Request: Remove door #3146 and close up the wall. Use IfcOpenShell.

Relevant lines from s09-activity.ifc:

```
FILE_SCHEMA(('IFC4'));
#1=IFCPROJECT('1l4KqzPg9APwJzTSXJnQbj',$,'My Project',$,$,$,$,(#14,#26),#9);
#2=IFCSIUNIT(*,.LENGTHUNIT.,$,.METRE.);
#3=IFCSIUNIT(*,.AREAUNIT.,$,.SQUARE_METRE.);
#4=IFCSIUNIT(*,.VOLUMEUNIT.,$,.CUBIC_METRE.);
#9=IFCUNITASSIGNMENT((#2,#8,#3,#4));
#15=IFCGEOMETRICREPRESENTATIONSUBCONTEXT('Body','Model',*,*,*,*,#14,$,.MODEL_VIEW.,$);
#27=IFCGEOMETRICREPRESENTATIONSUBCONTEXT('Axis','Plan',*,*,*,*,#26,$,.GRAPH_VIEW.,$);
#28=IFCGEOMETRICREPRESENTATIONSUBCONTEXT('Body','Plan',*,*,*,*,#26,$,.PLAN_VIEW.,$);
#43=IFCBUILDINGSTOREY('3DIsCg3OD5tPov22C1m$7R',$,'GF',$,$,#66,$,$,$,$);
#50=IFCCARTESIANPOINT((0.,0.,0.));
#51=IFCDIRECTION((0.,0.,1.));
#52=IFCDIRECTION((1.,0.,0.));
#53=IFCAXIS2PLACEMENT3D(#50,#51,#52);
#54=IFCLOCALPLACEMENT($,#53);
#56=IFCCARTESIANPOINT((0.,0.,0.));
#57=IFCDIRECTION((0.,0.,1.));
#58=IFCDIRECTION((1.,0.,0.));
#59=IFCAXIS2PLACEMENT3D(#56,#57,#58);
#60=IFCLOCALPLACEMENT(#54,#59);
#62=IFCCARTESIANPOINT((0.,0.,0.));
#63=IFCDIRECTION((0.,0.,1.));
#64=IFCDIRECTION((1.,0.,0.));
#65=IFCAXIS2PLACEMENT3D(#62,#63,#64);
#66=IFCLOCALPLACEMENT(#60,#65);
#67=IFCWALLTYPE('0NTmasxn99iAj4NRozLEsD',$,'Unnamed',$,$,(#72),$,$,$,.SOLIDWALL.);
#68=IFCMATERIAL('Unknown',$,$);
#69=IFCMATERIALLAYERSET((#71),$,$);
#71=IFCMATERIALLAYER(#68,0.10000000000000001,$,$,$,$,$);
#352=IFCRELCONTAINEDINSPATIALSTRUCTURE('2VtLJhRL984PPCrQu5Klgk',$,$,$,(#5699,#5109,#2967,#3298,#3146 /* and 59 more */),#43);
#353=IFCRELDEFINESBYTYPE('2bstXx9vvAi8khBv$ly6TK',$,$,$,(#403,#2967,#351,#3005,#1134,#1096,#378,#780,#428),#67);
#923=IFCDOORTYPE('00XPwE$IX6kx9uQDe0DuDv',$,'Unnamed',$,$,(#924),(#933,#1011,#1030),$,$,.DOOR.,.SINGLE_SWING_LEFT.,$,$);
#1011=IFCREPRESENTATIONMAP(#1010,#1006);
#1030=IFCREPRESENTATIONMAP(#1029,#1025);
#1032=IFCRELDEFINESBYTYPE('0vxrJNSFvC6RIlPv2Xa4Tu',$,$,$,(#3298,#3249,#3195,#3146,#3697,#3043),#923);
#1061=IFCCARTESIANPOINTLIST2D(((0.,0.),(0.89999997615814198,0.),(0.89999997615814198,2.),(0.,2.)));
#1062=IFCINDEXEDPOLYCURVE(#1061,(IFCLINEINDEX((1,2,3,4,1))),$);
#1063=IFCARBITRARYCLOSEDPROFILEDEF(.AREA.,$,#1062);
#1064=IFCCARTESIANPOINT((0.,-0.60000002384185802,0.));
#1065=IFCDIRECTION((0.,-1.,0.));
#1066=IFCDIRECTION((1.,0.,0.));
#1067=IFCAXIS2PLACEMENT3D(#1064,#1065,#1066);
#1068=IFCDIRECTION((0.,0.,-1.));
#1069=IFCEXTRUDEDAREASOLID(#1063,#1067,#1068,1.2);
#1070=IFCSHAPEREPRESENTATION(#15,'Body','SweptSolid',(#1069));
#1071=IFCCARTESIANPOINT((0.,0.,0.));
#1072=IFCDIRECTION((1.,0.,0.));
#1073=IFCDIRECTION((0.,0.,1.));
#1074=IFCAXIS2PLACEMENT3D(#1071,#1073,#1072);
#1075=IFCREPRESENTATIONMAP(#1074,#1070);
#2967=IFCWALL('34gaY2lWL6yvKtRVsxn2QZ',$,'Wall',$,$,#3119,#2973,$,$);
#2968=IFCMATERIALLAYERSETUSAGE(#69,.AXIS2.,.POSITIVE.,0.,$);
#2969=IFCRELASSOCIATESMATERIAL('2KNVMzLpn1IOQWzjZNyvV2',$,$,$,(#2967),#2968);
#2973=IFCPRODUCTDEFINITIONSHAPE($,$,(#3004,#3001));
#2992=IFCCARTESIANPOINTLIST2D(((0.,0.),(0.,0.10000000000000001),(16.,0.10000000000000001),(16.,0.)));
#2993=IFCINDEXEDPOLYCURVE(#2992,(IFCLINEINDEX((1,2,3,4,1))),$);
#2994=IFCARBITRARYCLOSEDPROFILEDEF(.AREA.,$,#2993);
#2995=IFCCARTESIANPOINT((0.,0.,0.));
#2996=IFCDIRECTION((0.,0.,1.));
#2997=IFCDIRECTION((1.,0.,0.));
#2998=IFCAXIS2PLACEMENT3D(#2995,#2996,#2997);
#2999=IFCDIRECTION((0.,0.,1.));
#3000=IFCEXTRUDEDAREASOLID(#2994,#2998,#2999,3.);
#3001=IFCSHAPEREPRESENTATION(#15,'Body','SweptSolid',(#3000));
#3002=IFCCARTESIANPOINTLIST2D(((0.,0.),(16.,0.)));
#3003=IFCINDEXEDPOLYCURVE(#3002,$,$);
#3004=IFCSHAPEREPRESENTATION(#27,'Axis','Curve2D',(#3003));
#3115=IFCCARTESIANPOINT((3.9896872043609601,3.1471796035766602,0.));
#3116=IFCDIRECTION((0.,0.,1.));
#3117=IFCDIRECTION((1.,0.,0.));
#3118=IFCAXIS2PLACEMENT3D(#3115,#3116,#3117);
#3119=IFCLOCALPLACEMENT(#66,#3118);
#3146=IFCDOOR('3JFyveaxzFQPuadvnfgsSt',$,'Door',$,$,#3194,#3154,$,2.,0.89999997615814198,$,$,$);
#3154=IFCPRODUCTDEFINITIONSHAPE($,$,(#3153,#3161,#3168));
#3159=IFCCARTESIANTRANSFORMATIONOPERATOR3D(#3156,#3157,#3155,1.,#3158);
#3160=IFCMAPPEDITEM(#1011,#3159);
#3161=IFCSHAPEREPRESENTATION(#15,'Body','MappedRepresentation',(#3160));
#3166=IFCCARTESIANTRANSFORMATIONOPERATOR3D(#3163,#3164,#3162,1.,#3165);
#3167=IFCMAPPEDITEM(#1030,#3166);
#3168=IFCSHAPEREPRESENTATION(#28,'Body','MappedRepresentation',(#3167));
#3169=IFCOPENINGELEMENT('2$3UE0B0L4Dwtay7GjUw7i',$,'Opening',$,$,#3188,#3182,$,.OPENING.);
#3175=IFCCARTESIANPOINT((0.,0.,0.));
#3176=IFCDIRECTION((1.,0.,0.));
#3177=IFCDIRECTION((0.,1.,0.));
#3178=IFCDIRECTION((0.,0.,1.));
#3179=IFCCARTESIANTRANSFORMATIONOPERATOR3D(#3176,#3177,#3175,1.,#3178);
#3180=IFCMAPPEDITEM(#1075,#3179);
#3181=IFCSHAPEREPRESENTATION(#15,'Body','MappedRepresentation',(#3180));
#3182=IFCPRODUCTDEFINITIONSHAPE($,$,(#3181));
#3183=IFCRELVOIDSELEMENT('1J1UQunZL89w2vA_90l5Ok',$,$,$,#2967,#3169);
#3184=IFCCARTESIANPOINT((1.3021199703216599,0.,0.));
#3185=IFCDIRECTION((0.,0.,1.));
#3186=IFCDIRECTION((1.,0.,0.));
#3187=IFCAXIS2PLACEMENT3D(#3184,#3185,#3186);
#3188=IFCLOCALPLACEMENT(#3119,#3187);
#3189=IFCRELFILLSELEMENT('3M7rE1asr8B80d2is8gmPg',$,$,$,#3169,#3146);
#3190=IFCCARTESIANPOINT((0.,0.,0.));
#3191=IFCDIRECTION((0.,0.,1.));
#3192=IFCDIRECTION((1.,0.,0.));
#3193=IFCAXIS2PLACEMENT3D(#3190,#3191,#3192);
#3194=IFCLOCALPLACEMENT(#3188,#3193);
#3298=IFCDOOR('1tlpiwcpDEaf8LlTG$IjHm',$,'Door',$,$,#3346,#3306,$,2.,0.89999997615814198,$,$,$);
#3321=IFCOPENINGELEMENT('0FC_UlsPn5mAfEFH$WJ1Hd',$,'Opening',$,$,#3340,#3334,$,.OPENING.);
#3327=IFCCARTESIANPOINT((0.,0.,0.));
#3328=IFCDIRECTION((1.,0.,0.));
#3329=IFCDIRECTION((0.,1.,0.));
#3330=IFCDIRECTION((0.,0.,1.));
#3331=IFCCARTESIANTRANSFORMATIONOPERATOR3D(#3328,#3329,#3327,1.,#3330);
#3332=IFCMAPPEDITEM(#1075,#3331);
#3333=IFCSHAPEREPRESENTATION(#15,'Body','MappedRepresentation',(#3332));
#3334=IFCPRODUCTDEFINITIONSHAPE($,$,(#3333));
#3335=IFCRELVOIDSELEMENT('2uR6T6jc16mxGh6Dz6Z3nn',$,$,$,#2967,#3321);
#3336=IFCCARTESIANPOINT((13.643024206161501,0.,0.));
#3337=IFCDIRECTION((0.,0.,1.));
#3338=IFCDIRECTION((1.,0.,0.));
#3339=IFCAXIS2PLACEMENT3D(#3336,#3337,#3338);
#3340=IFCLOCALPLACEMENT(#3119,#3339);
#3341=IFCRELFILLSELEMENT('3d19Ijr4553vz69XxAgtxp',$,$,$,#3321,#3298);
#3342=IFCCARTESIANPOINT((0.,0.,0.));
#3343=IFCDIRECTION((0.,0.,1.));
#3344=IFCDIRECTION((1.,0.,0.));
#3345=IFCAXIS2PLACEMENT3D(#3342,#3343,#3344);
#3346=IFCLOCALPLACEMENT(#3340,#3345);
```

```python
import ifcopenshell
import ifcopenshell.api.feature
import ifcopenshell.api.root
import ifcopenshell.geom
import ifcopenshell.util.shape

model = ifcopenshell.open("s09-activity.ifc")
settings = ifcopenshell.geom.settings()


def volume(element):
    """Net volume in cubic metres, openings subtracted."""
    shape = ifcopenshell.geom.create_shape(settings, element)
    return ifcopenshell.util.shape.get_volume(shape.geometry)


door = model.by_guid("3JFyveaxzFQPuadvnfgsSt")
opening = door.FillsVoids[0].RelatingOpeningElement
wall = opening.VoidsElements[0].RelatingBuildingElement
before = volume(wall)

ifcopenshell.api.root.remove_product(model, product=door)
ifcopenshell.api.feature.remove_feature(model, feature=opening)

after = volume(wall)

print(f"wall volume {before:.3f} -> {after:.3f} m3")

model.write("s09-activity_rev.ifc")
```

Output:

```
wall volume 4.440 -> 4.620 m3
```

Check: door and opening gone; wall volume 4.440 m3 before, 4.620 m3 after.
